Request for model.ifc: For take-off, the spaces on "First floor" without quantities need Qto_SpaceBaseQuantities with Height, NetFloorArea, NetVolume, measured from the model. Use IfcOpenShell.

First a look at what the model holds.

```python
import ifcopenshell
import ifcopenshell.util.element
import ifcopenshell.util.unit

model = ifcopenshell.open("model.ifc")
print(model.schema)
for unit_type in ("LENGTHUNIT", "AREAUNIT", "VOLUMEUNIT"):
    print(unit_type, ifcopenshell.util.unit.calculate_unit_scale(model, unit_type))
storey = next(s for s in model.by_type("IfcBuildingStorey") if s.Name == "First floor")
spaces = [e for e in ifcopenshell.util.element.get_decomposition(storey) if e.is_a("IfcSpace")]
for e in sorted(spaces, key=lambda e: e.id()):
    print(e.id(), e.is_a(), e.Name, list(ifcopenshell.util.element.get_psets(e, qtos_only=True)), sep=" | ")
```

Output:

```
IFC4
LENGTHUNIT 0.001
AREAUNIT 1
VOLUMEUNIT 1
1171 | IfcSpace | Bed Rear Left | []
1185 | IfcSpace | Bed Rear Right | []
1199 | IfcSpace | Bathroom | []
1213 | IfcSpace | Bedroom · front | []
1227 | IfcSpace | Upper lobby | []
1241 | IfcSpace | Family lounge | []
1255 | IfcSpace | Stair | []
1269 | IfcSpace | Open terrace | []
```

```python
import ifcopenshell
import ifcopenshell.api.pset
import ifcopenshell.geom
import ifcopenshell.util.element
import ifcopenshell.util.shape
import ifcopenshell.util.unit

model = ifcopenshell.open("model.ifc")
unit_scale = ifcopenshell.util.unit.calculate_unit_scale(model)
area_scale = ifcopenshell.util.unit.calculate_unit_scale(model, "AREAUNIT")
volume_scale = ifcopenshell.util.unit.calculate_unit_scale(model, "VOLUMEUNIT")
settings = ifcopenshell.geom.settings()

storey = next(s for s in model.by_type("IfcBuildingStorey") if s.Name == "First floor")
spaces = [e for e in ifcopenshell.util.element.get_decomposition(storey) if e.is_a("IfcSpace")]

for e in sorted(spaces, key=lambda e: e.id()):
    if ifcopenshell.util.element.get_psets(e, qtos_only=True, should_inherit=False):
        continue
    # Geometry comes back in metres, in the element's own axes.
    shape = ifcopenshell.geom.create_shape(settings, e)
    values = {
        "Height": ifcopenshell.util.shape.get_z(shape.geometry) / unit_scale,
        "NetFloorArea": ifcopenshell.util.shape.get_footprint_area(shape.geometry) / area_scale,
        "NetVolume": ifcopenshell.util.shape.get_volume(shape.geometry) / volume_scale,
    }
    qto = ifcopenshell.api.pset.add_qto(model, product=e, name="Qto_SpaceBaseQuantities")
    ifcopenshell.api.pset.edit_qto(model, qto=qto, properties=values)
    print(e.id(), {k: round(v, 3) for k, v in values.items()})

model.write("model_v2.ifc")
```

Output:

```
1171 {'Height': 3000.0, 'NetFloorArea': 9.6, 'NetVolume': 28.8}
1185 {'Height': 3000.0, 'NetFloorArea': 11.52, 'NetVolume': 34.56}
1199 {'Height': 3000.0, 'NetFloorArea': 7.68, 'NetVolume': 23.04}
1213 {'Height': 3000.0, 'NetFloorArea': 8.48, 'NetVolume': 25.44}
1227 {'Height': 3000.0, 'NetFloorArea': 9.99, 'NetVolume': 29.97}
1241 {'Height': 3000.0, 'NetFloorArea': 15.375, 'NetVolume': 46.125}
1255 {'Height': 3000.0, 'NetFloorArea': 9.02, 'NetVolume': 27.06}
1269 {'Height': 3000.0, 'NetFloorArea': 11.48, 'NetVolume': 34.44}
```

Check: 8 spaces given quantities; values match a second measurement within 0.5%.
